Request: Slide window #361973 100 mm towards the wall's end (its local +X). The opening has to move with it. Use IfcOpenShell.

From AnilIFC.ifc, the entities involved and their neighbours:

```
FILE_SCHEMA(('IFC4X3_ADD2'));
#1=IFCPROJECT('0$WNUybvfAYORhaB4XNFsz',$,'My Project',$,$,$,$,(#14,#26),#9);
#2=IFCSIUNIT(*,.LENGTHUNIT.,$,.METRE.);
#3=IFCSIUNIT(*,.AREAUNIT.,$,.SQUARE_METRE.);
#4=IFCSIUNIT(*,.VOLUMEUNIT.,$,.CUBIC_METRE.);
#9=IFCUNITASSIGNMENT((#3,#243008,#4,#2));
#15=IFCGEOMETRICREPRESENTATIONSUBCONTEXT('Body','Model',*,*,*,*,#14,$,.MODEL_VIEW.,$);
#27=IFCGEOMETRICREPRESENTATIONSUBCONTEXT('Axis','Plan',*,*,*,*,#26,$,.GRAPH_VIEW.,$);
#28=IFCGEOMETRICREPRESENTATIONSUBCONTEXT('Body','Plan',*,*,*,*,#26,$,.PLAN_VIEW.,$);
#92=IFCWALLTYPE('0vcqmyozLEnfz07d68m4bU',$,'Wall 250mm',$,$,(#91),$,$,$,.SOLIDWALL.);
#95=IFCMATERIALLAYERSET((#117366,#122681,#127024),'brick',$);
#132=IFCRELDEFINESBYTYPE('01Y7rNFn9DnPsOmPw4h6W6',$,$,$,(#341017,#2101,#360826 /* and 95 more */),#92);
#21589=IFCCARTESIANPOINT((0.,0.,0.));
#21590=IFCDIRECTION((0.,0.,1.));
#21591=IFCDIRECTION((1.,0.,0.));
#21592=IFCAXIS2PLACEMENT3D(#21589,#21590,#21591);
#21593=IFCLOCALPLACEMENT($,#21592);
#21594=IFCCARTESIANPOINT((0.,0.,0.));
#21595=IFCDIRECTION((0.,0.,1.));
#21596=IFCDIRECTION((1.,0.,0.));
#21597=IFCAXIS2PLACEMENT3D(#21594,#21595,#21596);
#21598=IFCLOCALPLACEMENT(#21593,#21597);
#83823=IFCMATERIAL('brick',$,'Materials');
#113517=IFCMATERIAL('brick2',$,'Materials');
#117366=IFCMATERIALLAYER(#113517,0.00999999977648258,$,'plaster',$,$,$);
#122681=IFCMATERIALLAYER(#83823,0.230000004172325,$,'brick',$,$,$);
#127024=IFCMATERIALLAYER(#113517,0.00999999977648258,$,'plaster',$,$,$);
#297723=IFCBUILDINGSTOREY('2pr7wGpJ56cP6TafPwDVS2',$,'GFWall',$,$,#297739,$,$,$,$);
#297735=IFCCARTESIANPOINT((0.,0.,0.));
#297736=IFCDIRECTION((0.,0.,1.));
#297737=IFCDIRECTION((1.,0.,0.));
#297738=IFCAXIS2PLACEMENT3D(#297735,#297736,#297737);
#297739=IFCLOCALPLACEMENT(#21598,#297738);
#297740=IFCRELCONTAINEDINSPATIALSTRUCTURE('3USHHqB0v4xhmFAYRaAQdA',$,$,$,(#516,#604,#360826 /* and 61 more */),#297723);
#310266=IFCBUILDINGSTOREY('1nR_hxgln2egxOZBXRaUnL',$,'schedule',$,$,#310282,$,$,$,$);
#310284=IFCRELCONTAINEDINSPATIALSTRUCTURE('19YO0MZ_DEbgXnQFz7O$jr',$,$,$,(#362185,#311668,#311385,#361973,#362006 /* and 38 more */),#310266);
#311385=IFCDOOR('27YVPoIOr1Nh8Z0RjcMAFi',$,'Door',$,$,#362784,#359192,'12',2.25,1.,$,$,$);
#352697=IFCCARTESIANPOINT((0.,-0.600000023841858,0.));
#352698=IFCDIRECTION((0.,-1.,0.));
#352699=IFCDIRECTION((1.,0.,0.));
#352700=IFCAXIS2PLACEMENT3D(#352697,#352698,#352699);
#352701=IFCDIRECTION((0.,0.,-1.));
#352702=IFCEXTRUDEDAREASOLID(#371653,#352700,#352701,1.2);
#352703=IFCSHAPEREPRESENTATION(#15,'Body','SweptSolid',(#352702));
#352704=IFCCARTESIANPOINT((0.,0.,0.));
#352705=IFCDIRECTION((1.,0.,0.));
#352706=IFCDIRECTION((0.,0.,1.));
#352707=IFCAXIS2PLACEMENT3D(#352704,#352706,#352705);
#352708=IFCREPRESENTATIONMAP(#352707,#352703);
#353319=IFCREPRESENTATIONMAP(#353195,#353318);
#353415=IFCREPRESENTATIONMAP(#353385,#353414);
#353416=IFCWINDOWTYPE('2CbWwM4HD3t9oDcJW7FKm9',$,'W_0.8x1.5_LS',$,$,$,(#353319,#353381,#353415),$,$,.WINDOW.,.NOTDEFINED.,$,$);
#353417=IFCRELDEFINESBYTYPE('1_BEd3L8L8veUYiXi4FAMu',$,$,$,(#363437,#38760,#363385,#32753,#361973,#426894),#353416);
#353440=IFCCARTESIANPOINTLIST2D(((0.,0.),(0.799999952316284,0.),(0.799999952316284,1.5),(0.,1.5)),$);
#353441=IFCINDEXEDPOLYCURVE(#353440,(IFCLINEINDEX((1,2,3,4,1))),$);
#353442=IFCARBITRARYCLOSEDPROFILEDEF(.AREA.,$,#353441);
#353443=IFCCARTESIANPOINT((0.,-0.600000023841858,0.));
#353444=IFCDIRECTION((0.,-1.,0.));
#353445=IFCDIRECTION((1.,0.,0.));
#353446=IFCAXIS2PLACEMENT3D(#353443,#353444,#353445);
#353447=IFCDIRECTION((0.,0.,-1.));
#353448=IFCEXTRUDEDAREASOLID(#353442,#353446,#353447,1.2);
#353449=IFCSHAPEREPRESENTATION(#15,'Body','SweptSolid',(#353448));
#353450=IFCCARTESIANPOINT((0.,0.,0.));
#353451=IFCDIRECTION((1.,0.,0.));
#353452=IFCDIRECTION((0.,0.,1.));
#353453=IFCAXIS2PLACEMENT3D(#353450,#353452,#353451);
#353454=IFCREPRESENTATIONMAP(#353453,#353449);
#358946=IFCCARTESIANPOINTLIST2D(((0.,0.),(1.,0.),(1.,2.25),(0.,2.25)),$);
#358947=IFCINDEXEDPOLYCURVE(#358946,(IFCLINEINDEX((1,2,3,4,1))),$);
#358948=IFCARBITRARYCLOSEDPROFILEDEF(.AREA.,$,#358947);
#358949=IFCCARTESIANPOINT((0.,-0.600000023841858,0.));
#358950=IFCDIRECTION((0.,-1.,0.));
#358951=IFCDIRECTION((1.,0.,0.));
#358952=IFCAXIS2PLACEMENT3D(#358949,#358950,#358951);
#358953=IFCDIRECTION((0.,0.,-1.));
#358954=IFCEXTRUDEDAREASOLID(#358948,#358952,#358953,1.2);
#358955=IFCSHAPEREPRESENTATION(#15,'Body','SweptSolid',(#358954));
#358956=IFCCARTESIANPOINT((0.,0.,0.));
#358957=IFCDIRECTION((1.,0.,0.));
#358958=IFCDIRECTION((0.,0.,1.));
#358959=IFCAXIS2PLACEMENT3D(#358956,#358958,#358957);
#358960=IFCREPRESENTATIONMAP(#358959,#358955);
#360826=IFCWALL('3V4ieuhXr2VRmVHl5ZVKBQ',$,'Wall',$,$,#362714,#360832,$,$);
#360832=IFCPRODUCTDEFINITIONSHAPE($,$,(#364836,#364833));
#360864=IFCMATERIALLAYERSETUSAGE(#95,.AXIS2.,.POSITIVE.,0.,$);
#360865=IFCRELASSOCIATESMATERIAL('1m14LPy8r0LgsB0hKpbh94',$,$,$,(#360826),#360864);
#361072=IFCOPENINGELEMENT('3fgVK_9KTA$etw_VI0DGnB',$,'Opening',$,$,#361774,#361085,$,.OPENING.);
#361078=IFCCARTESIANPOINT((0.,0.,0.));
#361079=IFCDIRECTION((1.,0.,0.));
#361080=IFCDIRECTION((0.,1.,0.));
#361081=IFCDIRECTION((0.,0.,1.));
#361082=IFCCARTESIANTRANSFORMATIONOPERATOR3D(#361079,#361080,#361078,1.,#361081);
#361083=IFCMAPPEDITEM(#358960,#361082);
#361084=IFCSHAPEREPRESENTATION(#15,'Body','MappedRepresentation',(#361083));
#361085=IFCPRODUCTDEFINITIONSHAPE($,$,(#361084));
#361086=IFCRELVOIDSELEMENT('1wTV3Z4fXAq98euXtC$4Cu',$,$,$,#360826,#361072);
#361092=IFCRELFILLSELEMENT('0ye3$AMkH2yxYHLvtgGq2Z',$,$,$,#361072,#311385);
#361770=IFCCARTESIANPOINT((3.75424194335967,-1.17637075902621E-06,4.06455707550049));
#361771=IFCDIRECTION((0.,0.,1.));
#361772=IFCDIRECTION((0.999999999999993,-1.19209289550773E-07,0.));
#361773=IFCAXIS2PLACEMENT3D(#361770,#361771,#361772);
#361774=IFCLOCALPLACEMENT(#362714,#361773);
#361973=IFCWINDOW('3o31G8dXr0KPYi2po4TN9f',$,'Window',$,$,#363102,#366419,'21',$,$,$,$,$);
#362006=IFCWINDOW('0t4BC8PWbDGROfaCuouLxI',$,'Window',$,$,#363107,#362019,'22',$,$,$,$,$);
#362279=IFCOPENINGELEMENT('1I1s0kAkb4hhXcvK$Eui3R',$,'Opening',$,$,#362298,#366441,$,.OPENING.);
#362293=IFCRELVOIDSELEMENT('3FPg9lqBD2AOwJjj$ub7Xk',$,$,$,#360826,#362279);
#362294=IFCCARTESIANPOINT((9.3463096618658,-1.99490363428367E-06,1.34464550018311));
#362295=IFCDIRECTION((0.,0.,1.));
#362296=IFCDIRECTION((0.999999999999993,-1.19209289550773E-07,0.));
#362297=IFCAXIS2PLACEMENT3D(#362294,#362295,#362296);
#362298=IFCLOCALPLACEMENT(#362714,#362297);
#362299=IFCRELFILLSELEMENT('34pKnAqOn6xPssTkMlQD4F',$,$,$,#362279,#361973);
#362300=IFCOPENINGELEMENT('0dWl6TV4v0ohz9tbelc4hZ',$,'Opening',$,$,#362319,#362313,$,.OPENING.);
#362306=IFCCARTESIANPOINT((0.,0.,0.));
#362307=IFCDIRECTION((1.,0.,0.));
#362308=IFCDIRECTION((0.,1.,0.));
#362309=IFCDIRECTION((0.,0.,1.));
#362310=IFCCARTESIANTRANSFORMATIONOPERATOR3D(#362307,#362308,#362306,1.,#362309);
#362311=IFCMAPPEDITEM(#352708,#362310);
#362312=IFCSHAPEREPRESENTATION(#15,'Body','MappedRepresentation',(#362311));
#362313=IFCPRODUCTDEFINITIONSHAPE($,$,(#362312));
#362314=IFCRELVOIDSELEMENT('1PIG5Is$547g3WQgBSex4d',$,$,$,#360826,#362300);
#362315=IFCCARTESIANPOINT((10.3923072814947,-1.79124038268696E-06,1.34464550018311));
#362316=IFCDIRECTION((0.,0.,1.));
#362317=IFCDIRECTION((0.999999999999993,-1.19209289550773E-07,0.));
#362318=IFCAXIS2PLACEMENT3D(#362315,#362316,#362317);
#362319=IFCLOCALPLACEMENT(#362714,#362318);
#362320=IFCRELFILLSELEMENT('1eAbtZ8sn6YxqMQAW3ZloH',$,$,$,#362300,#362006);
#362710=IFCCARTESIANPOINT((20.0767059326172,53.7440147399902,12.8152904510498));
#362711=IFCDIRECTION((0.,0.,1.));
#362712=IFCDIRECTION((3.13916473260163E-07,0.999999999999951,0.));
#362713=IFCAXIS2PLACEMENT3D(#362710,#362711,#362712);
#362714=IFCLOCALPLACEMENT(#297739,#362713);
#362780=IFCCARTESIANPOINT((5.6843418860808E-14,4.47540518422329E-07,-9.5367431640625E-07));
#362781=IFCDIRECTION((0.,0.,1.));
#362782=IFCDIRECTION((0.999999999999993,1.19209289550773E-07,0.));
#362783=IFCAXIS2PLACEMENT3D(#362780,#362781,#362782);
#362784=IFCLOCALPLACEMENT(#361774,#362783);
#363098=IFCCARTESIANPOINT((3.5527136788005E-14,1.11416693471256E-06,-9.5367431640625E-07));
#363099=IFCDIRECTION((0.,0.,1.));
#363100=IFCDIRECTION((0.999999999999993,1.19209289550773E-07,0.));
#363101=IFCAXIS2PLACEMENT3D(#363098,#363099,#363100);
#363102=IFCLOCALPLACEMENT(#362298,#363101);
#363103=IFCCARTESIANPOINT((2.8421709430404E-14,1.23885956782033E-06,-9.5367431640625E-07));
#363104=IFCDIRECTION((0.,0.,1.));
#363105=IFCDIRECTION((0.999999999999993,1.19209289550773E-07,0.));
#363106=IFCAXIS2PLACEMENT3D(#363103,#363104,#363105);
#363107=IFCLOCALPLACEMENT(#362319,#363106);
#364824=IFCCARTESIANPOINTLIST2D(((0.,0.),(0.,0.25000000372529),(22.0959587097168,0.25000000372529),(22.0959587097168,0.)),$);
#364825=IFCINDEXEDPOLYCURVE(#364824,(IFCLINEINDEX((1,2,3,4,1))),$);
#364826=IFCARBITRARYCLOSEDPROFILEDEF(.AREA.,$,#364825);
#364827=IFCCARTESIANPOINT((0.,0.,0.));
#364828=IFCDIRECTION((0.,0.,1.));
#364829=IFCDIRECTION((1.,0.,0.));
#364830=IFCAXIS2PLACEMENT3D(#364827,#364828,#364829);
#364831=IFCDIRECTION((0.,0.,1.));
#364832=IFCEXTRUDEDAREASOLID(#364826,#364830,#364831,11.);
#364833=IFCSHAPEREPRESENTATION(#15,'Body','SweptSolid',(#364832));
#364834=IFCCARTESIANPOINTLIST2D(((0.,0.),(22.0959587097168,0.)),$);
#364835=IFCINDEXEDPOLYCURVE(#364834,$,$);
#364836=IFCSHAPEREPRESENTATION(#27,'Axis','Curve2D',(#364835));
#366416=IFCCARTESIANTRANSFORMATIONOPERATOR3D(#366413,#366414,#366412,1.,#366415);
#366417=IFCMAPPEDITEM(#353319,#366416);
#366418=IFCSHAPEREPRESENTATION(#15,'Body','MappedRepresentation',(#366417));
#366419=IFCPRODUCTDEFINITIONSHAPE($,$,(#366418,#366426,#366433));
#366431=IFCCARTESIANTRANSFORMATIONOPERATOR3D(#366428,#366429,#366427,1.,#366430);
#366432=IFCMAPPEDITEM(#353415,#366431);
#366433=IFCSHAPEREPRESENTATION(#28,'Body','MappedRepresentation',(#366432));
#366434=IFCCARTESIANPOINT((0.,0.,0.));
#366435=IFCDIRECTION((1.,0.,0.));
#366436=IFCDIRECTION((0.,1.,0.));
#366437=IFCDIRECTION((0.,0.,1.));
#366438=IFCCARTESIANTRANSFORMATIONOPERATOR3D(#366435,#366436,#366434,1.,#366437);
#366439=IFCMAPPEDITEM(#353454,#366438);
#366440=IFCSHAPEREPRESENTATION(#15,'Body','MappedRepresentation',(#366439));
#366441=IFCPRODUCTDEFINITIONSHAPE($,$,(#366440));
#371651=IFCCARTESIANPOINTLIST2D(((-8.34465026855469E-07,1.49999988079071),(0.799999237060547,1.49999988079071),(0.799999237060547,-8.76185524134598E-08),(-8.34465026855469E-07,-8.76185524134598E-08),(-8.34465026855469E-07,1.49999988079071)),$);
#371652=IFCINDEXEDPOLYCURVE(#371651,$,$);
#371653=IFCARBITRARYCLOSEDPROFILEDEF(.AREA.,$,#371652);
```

```python
import ifcopenshell
import ifcopenshell.api.geometry
import ifcopenshell.util.placement
import ifcopenshell.util.unit

model = ifcopenshell.open("AnilIFC.ifc")
unit_scale = ifcopenshell.util.unit.calculate_unit_scale(model)

window = model.by_guid("3o31G8dXr0KPYi2po4TN9f")
opening = window.FillsVoids[0].RelatingOpeningElement
wall = opening.VoidsElements[0].RelatingBuildingElement

wall_matrix = ifcopenshell.util.placement.get_local_placement(wall.ObjectPlacement)
shift = wall_matrix[:3, 0] * 0.1 / unit_scale
before = ifcopenshell.util.placement.get_local_placement(window.ObjectPlacement)[:3, 3].copy()

# The window is placed relative to its opening, so it follows when the opening moves.
matrix = ifcopenshell.util.placement.get_local_placement(opening.ObjectPlacement)
matrix[:3, 3] += shift
ifcopenshell.api.geometry.edit_object_placement(
    model, product=opening, matrix=matrix, is_si=False, should_transform_children=True
)

after = ifcopenshell.util.placement.get_local_placement(window.ObjectPlacement)[:3, 3]
print("window moved by", (after - before).round(3) + 0.0)

model.write("AnilIFC_updated.ifc")
```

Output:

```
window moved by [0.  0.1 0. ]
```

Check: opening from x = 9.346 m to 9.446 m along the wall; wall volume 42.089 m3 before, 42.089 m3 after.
